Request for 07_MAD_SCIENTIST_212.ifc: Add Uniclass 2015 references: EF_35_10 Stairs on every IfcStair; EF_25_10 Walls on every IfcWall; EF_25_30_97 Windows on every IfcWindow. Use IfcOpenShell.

First a look at what the model holds.

```python
import ifcopenshell

model = ifcopenshell.open("07_MAD_SCIENTIST_212.ifc")
print(model.schema)
print("classifications:", [c.Name for c in model.by_type("IfcClassification")])
for ifc_class in ("IfcDoor", "IfcRoof", "IfcStair", "IfcWall", "IfcWindow"):
    print(ifc_class, len(model.by_type(ifc_class)))
```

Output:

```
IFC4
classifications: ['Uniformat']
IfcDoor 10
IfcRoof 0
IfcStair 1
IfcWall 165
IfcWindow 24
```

```python
import ifcopenshell
import ifcopenshell.api.classification

model = ifcopenshell.open("07_MAD_SCIENTIST_212.ifc")

system = ifcopenshell.api.classification.add_classification(model, classification="Uniclass 2015")

codes = {
    "IfcStair": ("EF_35_10", "Stairs"),
    "IfcWall": ("EF_25_10", "Walls"),
    "IfcWindow": ("EF_25_30_97", "Windows"),
}
for ifc_class, (code, name) in codes.items():
    products = model.by_type(ifc_class)
    ifcopenshell.api.classification.add_reference(
        model, products=products, classification=system, identification=code, name=name
    )
    print(code, len(products))

model.write("07_MAD_SCIENTIST_212_v2.ifc")
```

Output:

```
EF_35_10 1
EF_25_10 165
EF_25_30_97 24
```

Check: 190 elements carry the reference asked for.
